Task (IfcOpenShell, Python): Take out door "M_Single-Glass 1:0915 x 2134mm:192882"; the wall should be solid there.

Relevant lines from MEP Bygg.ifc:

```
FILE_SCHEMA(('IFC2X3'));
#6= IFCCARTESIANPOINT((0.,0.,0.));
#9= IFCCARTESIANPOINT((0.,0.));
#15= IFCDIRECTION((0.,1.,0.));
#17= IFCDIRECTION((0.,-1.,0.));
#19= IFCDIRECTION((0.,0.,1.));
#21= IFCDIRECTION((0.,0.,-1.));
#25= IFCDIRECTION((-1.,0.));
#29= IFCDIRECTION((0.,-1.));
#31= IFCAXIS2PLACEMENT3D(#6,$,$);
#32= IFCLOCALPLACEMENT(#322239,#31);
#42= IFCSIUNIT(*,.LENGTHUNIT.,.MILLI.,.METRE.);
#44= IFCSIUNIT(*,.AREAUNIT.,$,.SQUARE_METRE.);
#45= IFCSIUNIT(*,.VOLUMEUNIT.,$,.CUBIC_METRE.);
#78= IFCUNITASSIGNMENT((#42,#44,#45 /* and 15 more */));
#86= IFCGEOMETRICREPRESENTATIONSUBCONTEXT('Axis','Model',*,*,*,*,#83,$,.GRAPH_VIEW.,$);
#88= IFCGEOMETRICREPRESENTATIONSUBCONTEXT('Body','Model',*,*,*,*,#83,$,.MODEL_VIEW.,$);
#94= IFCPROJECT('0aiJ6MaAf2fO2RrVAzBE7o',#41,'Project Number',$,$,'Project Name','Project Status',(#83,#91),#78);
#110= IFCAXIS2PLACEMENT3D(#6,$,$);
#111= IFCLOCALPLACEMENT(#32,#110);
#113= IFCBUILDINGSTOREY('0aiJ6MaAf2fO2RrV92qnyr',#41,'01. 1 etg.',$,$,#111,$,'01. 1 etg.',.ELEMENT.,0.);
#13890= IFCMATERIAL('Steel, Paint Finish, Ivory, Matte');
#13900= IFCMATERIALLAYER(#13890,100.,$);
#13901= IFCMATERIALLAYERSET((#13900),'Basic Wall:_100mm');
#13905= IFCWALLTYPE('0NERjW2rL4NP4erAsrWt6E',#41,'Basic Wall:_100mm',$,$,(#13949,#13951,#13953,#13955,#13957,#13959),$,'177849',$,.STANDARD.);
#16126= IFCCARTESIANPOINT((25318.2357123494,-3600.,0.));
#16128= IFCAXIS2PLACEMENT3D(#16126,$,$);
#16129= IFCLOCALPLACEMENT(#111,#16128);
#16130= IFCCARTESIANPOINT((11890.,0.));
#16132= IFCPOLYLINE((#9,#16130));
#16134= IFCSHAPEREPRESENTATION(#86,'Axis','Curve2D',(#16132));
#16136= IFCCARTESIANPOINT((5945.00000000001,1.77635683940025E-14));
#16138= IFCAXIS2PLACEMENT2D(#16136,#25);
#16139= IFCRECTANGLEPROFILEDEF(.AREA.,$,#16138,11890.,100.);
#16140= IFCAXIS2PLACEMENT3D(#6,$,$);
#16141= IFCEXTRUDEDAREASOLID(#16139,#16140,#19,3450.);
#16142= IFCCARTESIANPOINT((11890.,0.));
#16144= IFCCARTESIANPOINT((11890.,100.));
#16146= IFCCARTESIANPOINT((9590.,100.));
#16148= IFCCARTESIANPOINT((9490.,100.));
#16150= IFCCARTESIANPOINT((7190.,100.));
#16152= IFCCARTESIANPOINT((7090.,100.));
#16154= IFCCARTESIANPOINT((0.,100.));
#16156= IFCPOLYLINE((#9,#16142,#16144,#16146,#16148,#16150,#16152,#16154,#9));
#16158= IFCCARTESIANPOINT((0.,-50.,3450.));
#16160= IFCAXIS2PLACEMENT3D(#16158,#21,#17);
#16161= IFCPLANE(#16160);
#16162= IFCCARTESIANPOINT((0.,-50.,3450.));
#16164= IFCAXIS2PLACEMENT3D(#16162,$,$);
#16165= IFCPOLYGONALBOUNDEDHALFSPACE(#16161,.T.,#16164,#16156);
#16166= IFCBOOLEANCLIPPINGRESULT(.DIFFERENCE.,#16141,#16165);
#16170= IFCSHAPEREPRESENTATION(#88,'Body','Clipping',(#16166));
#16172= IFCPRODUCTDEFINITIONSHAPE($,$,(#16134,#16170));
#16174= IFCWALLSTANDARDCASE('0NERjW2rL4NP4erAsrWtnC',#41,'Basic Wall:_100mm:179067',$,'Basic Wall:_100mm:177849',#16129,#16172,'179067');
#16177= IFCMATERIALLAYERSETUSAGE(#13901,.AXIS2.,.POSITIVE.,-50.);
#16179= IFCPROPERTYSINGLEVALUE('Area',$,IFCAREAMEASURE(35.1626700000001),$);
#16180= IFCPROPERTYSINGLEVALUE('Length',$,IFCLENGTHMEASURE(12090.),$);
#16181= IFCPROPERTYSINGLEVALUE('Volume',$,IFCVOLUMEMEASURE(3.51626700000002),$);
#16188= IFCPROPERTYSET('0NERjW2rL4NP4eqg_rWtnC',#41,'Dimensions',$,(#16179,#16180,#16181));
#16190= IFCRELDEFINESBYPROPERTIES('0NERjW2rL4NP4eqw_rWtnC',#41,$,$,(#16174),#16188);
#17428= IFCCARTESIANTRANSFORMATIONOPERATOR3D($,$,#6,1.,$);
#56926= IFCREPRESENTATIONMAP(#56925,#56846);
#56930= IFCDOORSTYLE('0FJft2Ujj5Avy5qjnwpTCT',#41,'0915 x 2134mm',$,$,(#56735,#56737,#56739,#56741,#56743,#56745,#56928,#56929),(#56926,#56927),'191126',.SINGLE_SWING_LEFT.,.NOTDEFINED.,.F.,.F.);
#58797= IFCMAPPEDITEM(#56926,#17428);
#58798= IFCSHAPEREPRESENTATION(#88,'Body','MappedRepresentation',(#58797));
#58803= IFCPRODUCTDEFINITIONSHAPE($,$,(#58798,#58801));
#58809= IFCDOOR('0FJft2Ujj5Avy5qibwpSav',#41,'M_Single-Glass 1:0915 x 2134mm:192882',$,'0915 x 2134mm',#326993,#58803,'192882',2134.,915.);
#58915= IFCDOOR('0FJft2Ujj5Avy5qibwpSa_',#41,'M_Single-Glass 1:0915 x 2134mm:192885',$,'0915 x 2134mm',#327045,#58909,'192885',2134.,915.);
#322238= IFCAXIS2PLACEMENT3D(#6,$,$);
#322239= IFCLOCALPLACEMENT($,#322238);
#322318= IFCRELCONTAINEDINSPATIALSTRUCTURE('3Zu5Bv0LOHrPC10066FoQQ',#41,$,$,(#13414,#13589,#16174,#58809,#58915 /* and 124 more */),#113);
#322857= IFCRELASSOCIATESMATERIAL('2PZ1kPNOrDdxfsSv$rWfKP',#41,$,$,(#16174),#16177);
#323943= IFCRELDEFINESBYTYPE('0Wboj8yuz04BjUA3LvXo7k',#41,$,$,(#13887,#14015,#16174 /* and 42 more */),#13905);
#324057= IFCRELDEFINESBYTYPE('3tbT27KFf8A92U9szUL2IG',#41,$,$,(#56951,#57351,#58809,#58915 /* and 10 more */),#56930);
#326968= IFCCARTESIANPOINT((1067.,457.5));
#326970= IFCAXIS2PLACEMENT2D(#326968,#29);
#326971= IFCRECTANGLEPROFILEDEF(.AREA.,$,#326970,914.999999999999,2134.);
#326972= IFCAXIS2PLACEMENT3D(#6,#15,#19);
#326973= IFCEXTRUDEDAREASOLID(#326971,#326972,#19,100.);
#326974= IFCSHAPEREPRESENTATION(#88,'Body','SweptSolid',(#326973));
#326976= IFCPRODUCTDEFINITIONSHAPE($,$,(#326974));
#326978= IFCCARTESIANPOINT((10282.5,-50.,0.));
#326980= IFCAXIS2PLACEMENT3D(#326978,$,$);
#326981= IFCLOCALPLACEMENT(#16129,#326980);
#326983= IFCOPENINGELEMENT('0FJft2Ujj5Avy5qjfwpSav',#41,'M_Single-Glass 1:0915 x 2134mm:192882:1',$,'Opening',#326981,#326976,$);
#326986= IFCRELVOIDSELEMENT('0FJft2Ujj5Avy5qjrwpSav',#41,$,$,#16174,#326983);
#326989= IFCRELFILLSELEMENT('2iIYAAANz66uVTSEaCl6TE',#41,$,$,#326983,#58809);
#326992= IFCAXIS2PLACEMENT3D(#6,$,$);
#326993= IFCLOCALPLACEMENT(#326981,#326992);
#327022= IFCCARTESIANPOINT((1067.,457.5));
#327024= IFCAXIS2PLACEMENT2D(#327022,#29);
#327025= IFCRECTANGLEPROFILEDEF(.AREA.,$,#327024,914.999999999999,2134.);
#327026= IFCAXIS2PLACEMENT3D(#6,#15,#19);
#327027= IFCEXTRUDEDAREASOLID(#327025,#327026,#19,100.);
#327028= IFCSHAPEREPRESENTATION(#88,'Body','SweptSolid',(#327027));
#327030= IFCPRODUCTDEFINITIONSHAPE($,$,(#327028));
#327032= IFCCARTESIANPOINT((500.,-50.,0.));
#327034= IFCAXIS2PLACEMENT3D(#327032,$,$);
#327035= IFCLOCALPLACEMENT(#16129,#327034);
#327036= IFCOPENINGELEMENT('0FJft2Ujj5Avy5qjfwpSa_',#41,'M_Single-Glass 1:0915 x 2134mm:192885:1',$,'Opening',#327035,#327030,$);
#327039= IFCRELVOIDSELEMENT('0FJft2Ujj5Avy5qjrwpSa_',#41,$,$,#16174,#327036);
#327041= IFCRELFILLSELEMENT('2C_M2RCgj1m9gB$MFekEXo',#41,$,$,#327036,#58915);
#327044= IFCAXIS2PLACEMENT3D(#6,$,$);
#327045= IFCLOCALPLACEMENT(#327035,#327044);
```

```python
import ifcopenshell
import ifcopenshell.api.feature
import ifcopenshell.api.pset
import ifcopenshell.api.root
import ifcopenshell.geom
import ifcopenshell.util.element
import ifcopenshell.util.shape
import ifcopenshell.util.unit

model = ifcopenshell.open("MEP Bygg.ifc")
area_scale = ifcopenshell.util.unit.calculate_unit_scale(model, "AREAUNIT")
volume_scale = ifcopenshell.util.unit.calculate_unit_scale(model, "VOLUMEUNIT")
settings = ifcopenshell.geom.settings()


def volume(element):
    """Net volume in cubic metres, openings subtracted."""
    shape = ifcopenshell.geom.create_shape(settings, element)
    return ifcopenshell.util.shape.get_volume(shape.geometry)


door = model.by_guid("0FJft2Ujj5Avy5qibwpSav")
opening = door.FillsVoids[0].RelatingOpeningElement
wall = opening.VoidsElements[0].RelatingBuildingElement
before = volume(wall)

ifcopenshell.api.root.remove_product(model, product=door)
ifcopenshell.api.feature.remove_feature(model, feature=opening)

after = volume(wall)
thickness = 0.1  # wall thickness in metres

# Update the wall's stored quantities.
pset = model.by_id(ifcopenshell.util.element.get_pset(wall, "Dimensions", should_inherit=False)["id"])
ifcopenshell.api.pset.edit_pset(model, pset=pset, properties={
    "Area": model.create_entity("IfcAreaMeasure", after / thickness / area_scale),
    "Volume": model.create_entity("IfcVolumeMeasure", after / volume_scale),
})

print(f"wall volume {before:.3f} -> {after:.3f} m3")

model.write("MEP Bygg-out.ifc")
```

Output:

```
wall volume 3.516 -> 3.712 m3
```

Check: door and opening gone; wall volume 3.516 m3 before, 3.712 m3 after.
